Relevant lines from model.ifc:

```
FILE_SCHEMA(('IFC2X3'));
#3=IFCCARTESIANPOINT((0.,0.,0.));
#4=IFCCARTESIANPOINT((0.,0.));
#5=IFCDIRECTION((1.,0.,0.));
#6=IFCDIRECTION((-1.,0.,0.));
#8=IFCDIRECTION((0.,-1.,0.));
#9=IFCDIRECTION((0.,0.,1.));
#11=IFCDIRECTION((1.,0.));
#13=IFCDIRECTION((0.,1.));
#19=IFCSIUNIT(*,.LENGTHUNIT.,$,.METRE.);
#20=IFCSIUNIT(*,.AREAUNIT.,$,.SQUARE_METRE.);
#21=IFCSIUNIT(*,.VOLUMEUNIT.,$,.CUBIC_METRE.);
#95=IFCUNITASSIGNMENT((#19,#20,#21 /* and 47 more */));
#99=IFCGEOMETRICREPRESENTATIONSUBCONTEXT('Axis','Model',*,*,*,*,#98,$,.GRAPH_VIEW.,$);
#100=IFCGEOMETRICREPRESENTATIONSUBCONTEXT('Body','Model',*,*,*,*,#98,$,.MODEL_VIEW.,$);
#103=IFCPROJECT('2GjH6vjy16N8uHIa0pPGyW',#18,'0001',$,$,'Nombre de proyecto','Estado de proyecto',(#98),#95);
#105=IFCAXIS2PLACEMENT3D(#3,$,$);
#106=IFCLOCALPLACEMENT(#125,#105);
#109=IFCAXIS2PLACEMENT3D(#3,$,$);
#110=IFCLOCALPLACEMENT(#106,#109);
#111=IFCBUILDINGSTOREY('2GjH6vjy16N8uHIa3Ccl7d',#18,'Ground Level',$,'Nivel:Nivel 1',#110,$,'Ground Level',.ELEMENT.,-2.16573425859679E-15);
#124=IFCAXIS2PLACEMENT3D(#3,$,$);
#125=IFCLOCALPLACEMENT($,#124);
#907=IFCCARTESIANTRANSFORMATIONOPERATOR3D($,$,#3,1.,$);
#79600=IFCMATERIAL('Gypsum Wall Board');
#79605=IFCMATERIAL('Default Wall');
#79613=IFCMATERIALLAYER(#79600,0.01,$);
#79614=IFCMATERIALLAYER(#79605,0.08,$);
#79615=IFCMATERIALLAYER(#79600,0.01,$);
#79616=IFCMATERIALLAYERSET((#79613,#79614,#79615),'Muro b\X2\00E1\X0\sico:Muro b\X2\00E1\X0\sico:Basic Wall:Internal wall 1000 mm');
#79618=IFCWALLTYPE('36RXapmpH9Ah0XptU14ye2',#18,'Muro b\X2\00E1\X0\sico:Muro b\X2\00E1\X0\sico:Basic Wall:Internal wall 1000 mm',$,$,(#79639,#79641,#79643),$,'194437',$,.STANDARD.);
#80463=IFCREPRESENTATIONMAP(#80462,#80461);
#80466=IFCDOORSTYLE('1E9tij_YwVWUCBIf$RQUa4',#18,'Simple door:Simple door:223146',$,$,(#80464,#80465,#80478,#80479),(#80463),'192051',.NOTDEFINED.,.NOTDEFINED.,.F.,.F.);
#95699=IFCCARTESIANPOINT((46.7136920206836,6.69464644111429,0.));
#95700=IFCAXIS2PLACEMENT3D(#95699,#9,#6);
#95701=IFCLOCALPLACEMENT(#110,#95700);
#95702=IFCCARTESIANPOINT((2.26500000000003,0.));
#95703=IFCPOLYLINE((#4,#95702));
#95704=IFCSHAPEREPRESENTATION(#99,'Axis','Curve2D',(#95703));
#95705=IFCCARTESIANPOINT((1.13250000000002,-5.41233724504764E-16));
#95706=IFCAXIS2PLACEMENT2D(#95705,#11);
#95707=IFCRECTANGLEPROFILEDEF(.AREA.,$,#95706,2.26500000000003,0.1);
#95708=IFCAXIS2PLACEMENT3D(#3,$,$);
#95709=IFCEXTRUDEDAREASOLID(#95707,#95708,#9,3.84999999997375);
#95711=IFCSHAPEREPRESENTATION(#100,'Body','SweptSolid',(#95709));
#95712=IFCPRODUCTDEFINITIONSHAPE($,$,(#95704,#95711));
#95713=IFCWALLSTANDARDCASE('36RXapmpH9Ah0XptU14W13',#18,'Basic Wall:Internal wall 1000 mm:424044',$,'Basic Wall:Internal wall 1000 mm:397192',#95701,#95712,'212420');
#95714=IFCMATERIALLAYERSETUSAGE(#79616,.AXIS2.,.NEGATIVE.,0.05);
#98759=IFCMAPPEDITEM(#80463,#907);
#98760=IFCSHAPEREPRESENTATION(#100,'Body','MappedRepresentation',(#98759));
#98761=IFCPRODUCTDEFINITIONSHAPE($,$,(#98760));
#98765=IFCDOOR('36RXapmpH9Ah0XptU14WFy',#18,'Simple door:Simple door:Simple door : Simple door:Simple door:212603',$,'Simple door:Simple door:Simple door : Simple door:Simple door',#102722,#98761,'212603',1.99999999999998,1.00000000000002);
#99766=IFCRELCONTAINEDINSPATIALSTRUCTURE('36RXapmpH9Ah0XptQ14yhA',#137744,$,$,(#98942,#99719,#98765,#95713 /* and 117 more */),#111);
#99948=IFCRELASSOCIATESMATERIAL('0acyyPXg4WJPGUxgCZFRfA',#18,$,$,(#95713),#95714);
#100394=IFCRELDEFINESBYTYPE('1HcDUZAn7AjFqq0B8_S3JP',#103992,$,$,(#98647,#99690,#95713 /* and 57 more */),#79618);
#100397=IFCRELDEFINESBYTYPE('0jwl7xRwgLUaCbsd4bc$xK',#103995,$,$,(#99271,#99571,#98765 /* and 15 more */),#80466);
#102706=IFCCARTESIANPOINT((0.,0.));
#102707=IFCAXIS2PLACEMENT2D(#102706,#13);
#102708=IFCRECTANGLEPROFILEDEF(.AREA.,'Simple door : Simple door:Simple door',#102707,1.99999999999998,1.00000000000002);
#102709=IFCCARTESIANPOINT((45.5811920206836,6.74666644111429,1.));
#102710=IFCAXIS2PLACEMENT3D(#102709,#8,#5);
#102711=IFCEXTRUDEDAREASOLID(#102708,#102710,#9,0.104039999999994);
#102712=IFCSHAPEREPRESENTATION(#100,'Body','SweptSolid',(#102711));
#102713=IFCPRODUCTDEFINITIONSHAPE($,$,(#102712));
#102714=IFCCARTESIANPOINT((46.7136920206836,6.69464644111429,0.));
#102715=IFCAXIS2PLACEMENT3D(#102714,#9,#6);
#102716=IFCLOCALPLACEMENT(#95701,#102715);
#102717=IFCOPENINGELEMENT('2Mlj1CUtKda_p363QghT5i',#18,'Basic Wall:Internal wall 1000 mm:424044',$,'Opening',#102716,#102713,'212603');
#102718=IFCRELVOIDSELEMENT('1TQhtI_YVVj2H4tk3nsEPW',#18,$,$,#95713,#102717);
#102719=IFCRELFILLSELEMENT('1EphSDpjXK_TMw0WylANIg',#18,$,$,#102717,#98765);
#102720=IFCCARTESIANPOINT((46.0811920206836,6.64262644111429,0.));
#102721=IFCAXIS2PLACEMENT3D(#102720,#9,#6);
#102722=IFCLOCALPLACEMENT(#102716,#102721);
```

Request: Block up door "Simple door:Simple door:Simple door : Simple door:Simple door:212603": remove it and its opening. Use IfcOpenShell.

```python
import ifcopenshell
import ifcopenshell.api.feature
import ifcopenshell.api.root
import ifcopenshell.geom
import ifcopenshell.util.shape

model = ifcopenshell.open("model.ifc")
settings = ifcopenshell.geom.settings()


def volume(element):
    """Net volume in cubic metres, openings subtracted."""
    shape = ifcopenshell.geom.create_shape(settings, element)
    return ifcopenshell.util.shape.get_volume(shape.geometry)


door = model.by_id(98765)
opening = door.FillsVoids[0].RelatingOpeningElement
wall = opening.VoidsElements[0].RelatingBuildingElement
before = volume(wall)

ifcopenshell.api.root.remove_product(model, product=door)
ifcopenshell.api.feature.remove_feature(model, feature=opening)

after = volume(wall)

print(f"wall volume {before:.3f} -> {after:.3f} m3")

model.write("model_v2.ifc")
```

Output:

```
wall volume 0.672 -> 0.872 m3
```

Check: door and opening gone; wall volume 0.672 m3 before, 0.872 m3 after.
